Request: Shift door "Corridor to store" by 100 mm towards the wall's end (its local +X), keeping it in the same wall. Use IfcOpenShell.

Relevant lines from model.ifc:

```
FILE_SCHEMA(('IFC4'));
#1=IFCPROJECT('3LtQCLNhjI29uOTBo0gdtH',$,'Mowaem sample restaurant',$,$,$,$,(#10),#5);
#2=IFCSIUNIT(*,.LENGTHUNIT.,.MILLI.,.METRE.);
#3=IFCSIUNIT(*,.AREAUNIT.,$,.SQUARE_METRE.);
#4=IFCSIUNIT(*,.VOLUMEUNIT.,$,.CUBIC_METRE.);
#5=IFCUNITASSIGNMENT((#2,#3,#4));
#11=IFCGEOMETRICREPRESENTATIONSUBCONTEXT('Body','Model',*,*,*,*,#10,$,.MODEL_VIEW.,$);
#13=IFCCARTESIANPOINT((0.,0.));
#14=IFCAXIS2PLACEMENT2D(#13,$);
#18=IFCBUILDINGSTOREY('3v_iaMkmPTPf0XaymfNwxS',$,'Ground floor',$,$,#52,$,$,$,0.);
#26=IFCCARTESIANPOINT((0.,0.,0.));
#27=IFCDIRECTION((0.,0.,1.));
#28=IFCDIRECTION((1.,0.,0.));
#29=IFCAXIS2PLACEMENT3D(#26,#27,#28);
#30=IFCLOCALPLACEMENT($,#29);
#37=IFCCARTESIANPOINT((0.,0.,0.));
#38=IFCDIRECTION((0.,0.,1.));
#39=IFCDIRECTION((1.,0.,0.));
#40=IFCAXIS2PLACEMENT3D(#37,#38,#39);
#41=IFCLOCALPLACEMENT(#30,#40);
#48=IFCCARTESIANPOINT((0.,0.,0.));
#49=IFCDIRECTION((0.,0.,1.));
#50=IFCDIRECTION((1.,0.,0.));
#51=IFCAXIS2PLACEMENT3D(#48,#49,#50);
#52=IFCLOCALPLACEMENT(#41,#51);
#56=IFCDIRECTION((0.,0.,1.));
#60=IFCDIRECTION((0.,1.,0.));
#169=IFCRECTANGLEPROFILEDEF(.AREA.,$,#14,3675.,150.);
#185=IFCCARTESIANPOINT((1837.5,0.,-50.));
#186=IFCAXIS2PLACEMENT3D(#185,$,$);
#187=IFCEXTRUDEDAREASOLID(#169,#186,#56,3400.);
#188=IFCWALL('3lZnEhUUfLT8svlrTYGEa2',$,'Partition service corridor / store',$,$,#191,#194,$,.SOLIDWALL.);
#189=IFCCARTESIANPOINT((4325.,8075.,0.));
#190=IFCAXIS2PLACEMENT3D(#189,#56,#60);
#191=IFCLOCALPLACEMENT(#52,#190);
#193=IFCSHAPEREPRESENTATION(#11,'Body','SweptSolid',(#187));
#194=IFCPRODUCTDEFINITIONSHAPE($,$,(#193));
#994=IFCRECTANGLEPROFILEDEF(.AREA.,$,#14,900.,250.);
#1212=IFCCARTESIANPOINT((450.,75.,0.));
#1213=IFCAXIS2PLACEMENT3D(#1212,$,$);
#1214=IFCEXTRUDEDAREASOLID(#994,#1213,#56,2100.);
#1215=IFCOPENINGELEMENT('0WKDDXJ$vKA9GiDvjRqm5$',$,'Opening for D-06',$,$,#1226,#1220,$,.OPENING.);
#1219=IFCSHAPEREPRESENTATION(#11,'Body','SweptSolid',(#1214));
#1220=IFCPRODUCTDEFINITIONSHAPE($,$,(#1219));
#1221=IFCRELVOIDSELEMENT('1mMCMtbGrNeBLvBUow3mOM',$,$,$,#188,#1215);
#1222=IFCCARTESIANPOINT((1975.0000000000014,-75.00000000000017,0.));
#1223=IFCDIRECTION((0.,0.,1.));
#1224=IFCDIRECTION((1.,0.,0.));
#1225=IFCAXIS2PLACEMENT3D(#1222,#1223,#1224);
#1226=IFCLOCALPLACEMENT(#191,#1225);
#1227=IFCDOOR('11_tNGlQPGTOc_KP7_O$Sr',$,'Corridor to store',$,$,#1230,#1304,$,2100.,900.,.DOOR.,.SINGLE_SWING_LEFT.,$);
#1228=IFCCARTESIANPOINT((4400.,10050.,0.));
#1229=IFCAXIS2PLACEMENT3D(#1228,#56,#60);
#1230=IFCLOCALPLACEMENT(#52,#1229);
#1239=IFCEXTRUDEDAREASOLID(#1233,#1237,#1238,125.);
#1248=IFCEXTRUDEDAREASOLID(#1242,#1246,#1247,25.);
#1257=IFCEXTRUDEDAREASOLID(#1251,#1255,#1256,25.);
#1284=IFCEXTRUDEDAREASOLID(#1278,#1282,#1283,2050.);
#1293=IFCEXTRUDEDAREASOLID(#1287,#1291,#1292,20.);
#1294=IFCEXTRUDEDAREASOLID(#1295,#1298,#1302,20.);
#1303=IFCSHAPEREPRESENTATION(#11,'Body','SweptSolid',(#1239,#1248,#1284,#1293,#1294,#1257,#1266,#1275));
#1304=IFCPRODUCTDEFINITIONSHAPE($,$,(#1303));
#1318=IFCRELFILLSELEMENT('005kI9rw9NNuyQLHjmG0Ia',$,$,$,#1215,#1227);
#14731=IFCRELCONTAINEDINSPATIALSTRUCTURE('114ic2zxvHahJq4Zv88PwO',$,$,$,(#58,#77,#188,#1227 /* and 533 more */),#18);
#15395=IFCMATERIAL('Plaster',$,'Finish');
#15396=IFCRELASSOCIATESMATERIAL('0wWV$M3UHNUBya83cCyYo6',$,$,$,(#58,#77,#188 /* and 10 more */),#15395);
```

```python
import ifcopenshell
import ifcopenshell.api.geometry
import ifcopenshell.util.placement
import ifcopenshell.util.unit

model = ifcopenshell.open("model.ifc")
unit_scale = ifcopenshell.util.unit.calculate_unit_scale(model)

door = model.by_guid("11_tNGlQPGTOc_KP7_O$Sr")
opening = door.FillsVoids[0].RelatingOpeningElement
wall = opening.VoidsElements[0].RelatingBuildingElement

wall_matrix = ifcopenshell.util.placement.get_local_placement(wall.ObjectPlacement)
shift = wall_matrix[:3, 0] * 0.1 / unit_scale
before = ifcopenshell.util.placement.get_local_placement(door.ObjectPlacement)[:3, 3].copy()

# The door is not placed relative to its opening, so move both.
for product in (opening, door):
    matrix = ifcopenshell.util.placement.get_local_placement(product.ObjectPlacement)
    matrix[:3, 3] += shift
    ifcopenshell.api.geometry.edit_object_placement(model, product=product, matrix=matrix, is_si=False)

after = ifcopenshell.util.placement.get_local_placement(door.ObjectPlacement)[:3, 3]
print("door moved by", (after - before).round(3) + 0.0)

model.write("model_v2.ifc")
```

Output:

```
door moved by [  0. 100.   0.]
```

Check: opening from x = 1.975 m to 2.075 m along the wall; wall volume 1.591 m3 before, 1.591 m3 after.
